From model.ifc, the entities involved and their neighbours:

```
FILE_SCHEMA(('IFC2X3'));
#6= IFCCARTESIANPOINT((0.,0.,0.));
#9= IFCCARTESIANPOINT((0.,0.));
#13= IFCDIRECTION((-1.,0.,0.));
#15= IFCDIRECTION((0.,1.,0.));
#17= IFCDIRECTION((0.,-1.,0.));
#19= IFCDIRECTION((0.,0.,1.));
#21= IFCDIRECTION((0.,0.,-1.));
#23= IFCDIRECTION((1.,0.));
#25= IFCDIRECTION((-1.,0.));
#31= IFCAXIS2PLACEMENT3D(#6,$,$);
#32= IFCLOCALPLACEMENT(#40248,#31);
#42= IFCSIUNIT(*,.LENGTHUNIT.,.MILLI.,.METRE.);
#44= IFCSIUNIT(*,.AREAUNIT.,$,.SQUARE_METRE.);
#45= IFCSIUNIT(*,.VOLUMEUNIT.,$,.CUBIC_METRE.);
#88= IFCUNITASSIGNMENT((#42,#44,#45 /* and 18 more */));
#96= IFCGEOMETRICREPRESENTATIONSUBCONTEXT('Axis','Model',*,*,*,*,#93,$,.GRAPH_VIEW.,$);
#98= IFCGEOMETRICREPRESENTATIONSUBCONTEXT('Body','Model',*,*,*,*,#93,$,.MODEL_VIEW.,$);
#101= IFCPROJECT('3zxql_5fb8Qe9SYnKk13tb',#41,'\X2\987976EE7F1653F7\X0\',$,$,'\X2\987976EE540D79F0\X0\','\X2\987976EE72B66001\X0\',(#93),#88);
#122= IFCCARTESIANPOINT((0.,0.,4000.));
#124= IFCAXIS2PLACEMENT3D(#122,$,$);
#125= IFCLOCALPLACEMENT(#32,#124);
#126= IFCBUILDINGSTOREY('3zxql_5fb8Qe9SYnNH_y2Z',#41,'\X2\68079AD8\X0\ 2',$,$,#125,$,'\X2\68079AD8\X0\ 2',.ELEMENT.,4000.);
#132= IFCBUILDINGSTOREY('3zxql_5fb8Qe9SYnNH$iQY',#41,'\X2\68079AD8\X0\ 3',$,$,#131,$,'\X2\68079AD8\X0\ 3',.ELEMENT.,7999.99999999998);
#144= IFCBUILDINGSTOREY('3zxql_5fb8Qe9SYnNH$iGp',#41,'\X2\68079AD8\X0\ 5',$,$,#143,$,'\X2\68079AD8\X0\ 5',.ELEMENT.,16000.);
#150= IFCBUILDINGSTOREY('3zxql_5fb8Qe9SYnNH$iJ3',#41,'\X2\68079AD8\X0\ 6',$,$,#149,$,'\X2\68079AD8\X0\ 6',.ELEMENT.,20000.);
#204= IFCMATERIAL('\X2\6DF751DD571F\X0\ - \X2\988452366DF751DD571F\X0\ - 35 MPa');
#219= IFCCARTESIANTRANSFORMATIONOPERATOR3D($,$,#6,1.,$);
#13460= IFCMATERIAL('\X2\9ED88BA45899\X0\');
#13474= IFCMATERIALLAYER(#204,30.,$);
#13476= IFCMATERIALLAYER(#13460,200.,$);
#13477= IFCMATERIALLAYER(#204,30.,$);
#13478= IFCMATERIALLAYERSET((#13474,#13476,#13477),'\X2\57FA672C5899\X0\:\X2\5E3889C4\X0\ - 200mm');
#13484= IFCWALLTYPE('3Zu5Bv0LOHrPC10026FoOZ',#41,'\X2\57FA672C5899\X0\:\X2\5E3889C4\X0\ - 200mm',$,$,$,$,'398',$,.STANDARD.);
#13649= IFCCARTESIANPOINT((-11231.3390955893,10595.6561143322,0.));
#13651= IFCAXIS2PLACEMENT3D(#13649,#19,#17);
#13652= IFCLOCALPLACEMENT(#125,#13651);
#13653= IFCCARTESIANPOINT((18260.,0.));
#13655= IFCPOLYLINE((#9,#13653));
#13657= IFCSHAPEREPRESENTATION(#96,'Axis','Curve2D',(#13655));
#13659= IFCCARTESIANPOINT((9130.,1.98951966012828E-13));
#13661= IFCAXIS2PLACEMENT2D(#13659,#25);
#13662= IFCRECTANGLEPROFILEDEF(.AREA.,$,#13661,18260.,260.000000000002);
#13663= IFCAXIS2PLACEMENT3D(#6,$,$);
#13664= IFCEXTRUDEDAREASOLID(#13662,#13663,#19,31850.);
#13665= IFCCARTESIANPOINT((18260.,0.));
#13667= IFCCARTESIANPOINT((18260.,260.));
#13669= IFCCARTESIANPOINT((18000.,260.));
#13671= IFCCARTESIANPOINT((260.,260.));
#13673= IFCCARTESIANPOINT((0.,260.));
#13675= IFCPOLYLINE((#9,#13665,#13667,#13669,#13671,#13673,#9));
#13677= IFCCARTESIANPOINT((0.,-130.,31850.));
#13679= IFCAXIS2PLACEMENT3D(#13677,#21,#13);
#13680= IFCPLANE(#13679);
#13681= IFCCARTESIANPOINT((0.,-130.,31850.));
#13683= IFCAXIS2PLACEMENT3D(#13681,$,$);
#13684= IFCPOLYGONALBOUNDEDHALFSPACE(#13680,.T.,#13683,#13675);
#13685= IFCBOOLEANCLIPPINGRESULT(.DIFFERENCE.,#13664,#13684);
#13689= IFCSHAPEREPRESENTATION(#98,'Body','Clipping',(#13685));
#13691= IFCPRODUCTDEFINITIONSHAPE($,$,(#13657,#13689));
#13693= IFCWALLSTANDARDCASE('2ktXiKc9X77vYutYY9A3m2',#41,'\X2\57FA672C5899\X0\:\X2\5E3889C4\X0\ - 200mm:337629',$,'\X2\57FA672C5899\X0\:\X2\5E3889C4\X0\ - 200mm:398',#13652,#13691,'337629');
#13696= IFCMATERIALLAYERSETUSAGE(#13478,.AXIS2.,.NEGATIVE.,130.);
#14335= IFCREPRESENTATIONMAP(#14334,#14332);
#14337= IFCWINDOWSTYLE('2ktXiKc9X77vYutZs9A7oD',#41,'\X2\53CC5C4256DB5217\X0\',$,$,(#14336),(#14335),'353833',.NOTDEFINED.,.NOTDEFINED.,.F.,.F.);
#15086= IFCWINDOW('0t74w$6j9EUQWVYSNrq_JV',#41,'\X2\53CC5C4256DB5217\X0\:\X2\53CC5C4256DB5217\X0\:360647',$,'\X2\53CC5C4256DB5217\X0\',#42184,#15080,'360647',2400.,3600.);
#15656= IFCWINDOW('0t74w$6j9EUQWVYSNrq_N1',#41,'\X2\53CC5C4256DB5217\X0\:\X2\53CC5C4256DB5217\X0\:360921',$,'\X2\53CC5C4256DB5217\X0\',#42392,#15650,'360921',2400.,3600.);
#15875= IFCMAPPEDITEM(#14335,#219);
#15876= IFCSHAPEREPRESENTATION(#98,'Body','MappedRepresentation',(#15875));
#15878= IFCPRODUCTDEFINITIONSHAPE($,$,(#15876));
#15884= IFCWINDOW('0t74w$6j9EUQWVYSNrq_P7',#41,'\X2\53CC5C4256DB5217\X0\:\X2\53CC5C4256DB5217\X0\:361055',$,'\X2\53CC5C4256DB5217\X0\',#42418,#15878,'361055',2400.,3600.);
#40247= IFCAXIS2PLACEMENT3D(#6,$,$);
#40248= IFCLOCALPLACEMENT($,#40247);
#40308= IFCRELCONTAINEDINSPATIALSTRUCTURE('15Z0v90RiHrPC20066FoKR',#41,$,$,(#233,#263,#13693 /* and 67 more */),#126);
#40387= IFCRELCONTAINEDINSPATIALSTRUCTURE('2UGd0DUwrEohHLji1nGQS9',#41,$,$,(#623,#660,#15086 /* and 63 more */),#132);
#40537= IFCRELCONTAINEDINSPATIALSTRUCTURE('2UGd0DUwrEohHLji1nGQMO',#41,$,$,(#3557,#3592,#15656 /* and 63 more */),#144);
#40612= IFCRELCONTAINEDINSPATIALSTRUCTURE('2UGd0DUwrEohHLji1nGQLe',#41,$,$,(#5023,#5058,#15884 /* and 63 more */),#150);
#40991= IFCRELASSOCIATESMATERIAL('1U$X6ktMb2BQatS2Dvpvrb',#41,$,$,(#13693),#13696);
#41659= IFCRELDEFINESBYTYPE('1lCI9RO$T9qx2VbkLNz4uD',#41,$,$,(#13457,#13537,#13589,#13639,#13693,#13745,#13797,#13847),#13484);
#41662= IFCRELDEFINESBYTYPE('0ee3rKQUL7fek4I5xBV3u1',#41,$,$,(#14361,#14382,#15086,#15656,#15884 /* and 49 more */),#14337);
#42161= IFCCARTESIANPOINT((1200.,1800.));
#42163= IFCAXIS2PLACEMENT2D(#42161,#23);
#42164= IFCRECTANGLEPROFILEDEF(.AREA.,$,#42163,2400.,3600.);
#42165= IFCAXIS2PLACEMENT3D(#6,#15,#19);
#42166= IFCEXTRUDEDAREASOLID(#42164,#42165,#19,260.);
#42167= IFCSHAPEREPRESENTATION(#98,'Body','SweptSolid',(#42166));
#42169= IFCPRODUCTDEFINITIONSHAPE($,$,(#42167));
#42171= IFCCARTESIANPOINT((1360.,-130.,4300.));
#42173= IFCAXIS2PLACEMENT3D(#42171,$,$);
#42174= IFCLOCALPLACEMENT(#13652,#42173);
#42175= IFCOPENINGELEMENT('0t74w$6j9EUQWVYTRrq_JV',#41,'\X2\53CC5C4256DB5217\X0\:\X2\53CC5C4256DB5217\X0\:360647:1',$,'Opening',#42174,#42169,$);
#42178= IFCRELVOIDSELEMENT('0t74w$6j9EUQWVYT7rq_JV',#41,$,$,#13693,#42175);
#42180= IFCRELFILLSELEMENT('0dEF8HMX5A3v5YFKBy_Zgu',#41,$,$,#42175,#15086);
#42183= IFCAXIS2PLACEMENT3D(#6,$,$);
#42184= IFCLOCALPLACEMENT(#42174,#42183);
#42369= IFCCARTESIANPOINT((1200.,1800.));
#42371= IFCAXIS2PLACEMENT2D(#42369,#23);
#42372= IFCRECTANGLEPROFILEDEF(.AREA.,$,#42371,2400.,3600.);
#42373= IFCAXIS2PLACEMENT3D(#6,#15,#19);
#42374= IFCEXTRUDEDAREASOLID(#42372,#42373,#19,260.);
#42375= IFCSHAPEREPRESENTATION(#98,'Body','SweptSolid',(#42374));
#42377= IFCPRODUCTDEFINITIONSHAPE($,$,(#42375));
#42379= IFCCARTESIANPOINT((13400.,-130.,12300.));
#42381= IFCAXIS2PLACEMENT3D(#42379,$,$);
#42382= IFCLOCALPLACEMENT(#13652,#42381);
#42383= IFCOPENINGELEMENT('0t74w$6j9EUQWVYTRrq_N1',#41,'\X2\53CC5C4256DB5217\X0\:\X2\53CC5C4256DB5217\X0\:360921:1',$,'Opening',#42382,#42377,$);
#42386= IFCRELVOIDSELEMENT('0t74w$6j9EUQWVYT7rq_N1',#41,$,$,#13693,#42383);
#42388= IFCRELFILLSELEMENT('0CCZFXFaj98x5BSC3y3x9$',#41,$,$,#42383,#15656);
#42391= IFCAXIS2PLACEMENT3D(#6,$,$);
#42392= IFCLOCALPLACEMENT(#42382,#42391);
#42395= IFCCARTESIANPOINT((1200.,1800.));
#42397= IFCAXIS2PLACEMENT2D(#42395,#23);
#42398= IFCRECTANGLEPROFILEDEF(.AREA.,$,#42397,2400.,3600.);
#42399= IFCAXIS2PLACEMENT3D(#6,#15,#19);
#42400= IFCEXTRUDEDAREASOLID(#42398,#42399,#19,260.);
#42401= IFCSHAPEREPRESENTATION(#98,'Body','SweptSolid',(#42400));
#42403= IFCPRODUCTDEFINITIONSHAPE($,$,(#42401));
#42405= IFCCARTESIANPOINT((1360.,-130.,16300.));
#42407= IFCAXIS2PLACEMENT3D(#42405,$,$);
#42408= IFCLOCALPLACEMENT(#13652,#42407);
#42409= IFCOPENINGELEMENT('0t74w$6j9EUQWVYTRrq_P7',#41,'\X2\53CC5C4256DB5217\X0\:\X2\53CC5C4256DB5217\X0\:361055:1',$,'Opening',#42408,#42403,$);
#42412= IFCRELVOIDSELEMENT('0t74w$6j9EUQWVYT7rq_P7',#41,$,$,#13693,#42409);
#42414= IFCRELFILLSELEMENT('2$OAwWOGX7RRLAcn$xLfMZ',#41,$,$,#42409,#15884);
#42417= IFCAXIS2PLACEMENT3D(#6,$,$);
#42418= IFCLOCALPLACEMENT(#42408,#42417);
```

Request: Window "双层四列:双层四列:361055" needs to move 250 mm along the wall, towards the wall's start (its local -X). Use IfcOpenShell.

```python
import ifcopenshell
import ifcopenshell.api.geometry
import ifcopenshell.util.placement

model = ifcopenshell.open("model.ifc")

window = model.by_guid("0t74w$6j9EUQWVYSNrq_P7")
opening = window.FillsVoids[0].RelatingOpeningElement
wall = opening.VoidsElements[0].RelatingBuildingElement

wall_matrix = ifcopenshell.util.placement.get_local_placement(wall.ObjectPlacement)
shift = wall_matrix[:3, 0] * -250.0
before = ifcopenshell.util.placement.get_local_placement(window.ObjectPlacement)[:3, 3].copy()

# The window is placed relative to its opening, so it follows when the opening moves.
matrix = ifcopenshell.util.placement.get_local_placement(opening.ObjectPlacement)
matrix[:3, 3] += shift
ifcopenshell.api.geometry.edit_object_placement(
    model, product=opening, matrix=matrix, is_si=False, should_transform_children=True
)

after = ifcopenshell.util.placement.get_local_placement(window.ObjectPlacement)[:3, 3]
print("window moved by", (after - before).round(3) + 0.0)

model.write("model_updated.ifc")
```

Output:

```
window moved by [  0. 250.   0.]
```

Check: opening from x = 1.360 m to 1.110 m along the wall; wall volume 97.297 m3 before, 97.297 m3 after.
